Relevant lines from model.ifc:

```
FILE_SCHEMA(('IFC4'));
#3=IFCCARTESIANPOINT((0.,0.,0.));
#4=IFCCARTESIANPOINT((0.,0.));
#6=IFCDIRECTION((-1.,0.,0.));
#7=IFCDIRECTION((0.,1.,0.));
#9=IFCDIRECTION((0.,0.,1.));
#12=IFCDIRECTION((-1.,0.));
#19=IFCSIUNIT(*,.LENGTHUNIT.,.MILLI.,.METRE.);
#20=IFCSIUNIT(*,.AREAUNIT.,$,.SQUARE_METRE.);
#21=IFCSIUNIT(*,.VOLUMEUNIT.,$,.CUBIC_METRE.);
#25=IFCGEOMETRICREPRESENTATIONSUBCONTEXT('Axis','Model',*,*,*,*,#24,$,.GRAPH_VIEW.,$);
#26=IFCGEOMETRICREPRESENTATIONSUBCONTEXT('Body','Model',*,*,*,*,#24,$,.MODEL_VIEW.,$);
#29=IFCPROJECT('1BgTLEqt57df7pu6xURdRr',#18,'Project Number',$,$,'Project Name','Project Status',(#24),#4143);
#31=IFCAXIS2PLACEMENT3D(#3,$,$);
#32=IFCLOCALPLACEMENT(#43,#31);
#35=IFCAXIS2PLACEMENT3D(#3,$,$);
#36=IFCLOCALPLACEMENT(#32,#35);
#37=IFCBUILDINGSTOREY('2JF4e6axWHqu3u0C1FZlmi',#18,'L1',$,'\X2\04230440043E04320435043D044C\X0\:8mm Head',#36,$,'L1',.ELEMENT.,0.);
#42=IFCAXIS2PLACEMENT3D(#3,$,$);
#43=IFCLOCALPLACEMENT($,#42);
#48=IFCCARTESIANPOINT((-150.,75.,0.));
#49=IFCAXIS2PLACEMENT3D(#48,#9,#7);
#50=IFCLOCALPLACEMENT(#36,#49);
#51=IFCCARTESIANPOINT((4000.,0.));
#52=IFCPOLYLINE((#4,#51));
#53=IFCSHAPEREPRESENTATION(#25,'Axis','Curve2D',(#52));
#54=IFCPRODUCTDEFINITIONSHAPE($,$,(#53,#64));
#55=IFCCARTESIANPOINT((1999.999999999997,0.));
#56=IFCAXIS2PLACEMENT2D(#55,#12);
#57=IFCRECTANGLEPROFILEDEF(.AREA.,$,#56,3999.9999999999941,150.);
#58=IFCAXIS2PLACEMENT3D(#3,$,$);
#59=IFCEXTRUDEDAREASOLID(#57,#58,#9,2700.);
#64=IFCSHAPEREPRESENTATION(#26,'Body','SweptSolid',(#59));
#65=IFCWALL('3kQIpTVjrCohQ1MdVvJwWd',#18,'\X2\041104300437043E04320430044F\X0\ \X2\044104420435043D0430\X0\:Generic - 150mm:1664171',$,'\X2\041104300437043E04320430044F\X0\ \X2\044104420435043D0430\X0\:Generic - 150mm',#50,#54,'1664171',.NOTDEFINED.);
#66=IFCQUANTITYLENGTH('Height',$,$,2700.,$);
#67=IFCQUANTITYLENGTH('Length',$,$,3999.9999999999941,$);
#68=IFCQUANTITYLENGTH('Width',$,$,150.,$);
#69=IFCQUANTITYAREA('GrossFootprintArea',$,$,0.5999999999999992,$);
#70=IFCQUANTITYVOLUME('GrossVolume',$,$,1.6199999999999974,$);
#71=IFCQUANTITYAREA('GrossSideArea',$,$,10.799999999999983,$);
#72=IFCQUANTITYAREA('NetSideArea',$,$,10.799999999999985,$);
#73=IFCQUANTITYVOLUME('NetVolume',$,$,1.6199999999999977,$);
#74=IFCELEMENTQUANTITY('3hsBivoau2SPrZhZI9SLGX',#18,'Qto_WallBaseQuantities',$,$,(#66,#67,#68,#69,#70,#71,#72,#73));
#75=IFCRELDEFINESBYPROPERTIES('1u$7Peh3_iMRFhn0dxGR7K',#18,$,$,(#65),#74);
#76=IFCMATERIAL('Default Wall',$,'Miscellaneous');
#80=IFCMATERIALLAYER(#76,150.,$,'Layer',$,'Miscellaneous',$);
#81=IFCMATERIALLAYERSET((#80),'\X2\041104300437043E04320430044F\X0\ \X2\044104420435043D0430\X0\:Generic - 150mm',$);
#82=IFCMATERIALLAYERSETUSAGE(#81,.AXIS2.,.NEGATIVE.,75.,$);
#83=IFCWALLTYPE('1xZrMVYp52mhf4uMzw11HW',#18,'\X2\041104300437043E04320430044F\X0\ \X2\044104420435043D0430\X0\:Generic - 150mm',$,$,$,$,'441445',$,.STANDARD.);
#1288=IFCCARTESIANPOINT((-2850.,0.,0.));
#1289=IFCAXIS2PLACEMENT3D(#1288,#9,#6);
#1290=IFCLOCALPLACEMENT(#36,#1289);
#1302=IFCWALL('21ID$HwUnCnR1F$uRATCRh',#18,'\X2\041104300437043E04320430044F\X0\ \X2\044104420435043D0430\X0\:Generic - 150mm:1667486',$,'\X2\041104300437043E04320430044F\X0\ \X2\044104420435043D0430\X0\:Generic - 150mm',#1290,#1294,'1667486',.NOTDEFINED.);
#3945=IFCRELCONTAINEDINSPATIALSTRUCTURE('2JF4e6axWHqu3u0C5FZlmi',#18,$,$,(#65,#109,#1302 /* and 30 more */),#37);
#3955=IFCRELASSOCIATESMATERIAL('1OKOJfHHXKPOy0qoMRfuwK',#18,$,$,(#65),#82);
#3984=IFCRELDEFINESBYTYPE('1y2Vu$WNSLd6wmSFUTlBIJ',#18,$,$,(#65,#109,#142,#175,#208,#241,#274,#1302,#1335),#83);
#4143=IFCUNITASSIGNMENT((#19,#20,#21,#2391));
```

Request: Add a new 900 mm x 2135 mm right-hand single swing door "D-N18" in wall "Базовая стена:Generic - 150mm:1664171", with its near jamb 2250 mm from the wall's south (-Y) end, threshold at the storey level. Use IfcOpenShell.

```python
import numpy as np
import ifcopenshell
import ifcopenshell.api.feature
import ifcopenshell.api.geometry
import ifcopenshell.api.pset
import ifcopenshell.api.root
import ifcopenshell.api.spatial
import ifcopenshell.geom
import ifcopenshell.util.element
import ifcopenshell.util.placement
import ifcopenshell.util.representation
import ifcopenshell.util.shape
import ifcopenshell.util.unit

model = ifcopenshell.open("model.ifc")
unit_scale = ifcopenshell.util.unit.calculate_unit_scale(model)
area_scale = ifcopenshell.util.unit.calculate_unit_scale(model, "AREAUNIT")
volume_scale = ifcopenshell.util.unit.calculate_unit_scale(model, "VOLUMEUNIT")
settings = ifcopenshell.geom.settings()


def volume(element):
    """Net volume in cubic metres, openings subtracted."""
    shape = ifcopenshell.geom.create_shape(settings, element)
    return ifcopenshell.util.shape.get_volume(shape.geometry)


wall = model.by_guid("3kQIpTVjrCohQ1MdVvJwWd")
storey = ifcopenshell.util.element.get_container(wall, ifc_class="IfcBuildingStorey")
context = ifcopenshell.util.representation.get_context(model, "Model", "Body", "MODEL_VIEW")
before = volume(wall)

width, height, from_end, sill = 0.9, 2.135, 2.25, 0.0  # metres

# The wall runs along its own X axis, and the end named is its -X end.
wall_shape = ifcopenshell.geom.create_shape(settings, wall)
x, y, z = ifcopenshell.util.shape.get_vertices(wall_shape.geometry).T
start = x.min() + from_end
face, thickness = float(y.min()), float(y.max() - y.min())
wall_matrix = ifcopenshell.util.placement.get_local_placement(wall.ObjectPlacement)
level = ifcopenshell.util.placement.get_local_placement(storey.ObjectPlacement)[2, 3]


def in_wall(x, y):
    """Placement at x, y metres in the wall's axes, at sill height."""
    matrix = wall_matrix.copy()
    matrix[:, 3] = wall_matrix @ np.array([x / unit_scale, y / unit_scale, 0.0, 1.0])
    matrix[2, 3] = level + sill / unit_scale
    return matrix


# Opening: a box that overshoots both wall faces by 50 mm.
opening = ifcopenshell.api.root.create_entity(model, ifc_class="IfcOpeningElement", predefined_type="OPENING")
box = ifcopenshell.api.geometry.add_wall_representation(
    model, context=context, length=width, height=height, thickness=thickness + 0.1
)
ifcopenshell.api.geometry.assign_representation(model, product=opening, representation=box)
ifcopenshell.api.geometry.edit_object_placement(model, product=opening, matrix=in_wall(start, face - 0.05), is_si=False)
ifcopenshell.api.feature.add_feature(model, feature=opening, element=wall)

door = ifcopenshell.api.root.create_entity(model, ifc_class="IfcDoor", name="D-N18", predefined_type="DOOR")
door.OverallWidth, door.OverallHeight = width / unit_scale, height / unit_scale
door.OperationType = "SINGLE_SWING_RIGHT"
body = ifcopenshell.api.geometry.add_door_representation(
    model,
    context=context,
    overall_width=door.OverallWidth,
    overall_height=door.OverallHeight,
    operation_type="SINGLE_SWING_RIGHT",
    lining_properties={"LiningDepth": thickness / unit_scale, "ThresholdDepth": thickness / unit_scale},
)
ifcopenshell.api.geometry.assign_representation(model, product=door, representation=body)
ifcopenshell.api.spatial.assign_container(model, products=[door], relating_structure=storey)
ifcopenshell.api.feature.add_filling(model, opening=opening, element=door)

# The lining spans the wall, so the door starts at the wall face.
ifcopenshell.api.geometry.edit_object_placement(model, product=door, matrix=in_wall(start, face), is_si=False)

after = volume(wall)

# Update the wall's stored quantities.
qto = model.by_id(ifcopenshell.util.element.get_pset(wall, "Qto_WallBaseQuantities", should_inherit=False)["id"])
ifcopenshell.api.pset.edit_qto(model, qto=qto, properties={
    "NetSideArea": after / thickness / area_scale,
    "NetVolume": after / volume_scale,
})

print(f"wall volume {before:.3f} -> {after:.3f} m3")

model.write("model_updated.ifc")
```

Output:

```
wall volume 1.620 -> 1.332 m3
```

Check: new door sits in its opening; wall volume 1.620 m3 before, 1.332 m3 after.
